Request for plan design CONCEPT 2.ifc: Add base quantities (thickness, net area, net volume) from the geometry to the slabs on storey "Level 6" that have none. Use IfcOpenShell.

First a look at what the model holds.

```python
import ifcopenshell
import ifcopenshell.util.element
import ifcopenshell.util.unit

model = ifcopenshell.open("plan design CONCEPT 2.ifc")
print(model.schema)
for unit_type in ("LENGTHUNIT", "AREAUNIT", "VOLUMEUNIT"):
    print(unit_type, ifcopenshell.util.unit.calculate_unit_scale(model, unit_type))
storey = next(s for s in model.by_type("IfcBuildingStorey") if s.Name == "Level 6")
slabs = [e for e in ifcopenshell.util.element.get_decomposition(storey) if e.is_a("IfcSlab")]
for e in sorted(slabs, key=lambda e: e.id()):
    print(e.id(), e.is_a(), e.Name, list(ifcopenshell.util.element.get_psets(e, qtos_only=True)), sep=" | ")
```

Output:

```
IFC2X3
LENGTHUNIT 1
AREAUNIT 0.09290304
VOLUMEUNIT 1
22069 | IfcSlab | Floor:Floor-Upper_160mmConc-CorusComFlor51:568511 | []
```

```python
import ifcopenshell
import ifcopenshell.api.pset
import ifcopenshell.geom
import ifcopenshell.util.element
import ifcopenshell.util.shape
import ifcopenshell.util.unit

model = ifcopenshell.open("plan design CONCEPT 2.ifc")
unit_scale = ifcopenshell.util.unit.calculate_unit_scale(model)
area_scale = ifcopenshell.util.unit.calculate_unit_scale(model, "AREAUNIT")
volume_scale = ifcopenshell.util.unit.calculate_unit_scale(model, "VOLUMEUNIT")
settings = ifcopenshell.geom.settings()

storey = next(s for s in model.by_type("IfcBuildingStorey") if s.Name == "Level 6")
slabs = [e for e in ifcopenshell.util.element.get_decomposition(storey) if e.is_a("IfcSlab")]

for e in sorted(slabs, key=lambda e: e.id()):
    if ifcopenshell.util.element.get_psets(e, qtos_only=True, should_inherit=False):
        continue
    # Geometry comes back in metres, in the element's own axes.
    shape = ifcopenshell.geom.create_shape(settings, e)
    values = {
        "Width": ifcopenshell.util.shape.get_z(shape.geometry) / unit_scale,
        "NetArea": ifcopenshell.util.shape.get_footprint_area(shape.geometry) / area_scale,
        "NetVolume": ifcopenshell.util.shape.get_volume(shape.geometry) / volume_scale,
    }
    qto = ifcopenshell.api.pset.add_qto(model, product=e, name="BaseQuantities")
    ifcopenshell.api.pset.edit_qto(model, qto=qto, properties=values)
    print(e.id(), {k: round(v, 3) for k, v in values.items()})

model.write("plan design CONCEPT 2_rev.ifc")
```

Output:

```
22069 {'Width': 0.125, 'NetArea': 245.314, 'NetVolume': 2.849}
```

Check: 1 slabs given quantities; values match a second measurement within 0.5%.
